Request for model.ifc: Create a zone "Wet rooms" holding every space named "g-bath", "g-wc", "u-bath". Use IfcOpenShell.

First a look at what the model holds.

```python
import ifcopenshell

model = ifcopenshell.open("model.ifc")
print(model.schema)
seen = {}
for space in model.by_type("IfcSpace"):
    seen[space.LongName] = seen.get(space.LongName, 0) + 1
for name, count in sorted(seen.items(), key=str):
    print(count, "x", name)
print("zones:", [z.Name for z in model.by_type("IfcZone")][:20])
```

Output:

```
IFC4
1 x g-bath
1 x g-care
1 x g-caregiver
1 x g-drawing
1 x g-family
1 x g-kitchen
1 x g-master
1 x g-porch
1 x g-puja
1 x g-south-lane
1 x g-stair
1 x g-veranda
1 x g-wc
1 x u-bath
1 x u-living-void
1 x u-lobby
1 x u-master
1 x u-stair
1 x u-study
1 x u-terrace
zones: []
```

```python
import ifcopenshell
import ifcopenshell.api.group
import ifcopenshell.api.root

model = ifcopenshell.open("model.ifc")

names = {"g-bath", "g-wc", "u-bath"}
spaces = [s for s in model.by_type("IfcSpace") if s.LongName in names]

zone = ifcopenshell.api.root.create_entity(model, ifc_class="IfcZone", name="Wet rooms")
ifcopenshell.api.group.assign_group(model, products=spaces, group=zone)
print(len(spaces), "spaces in", zone.Name)

model.write("model_edited.ifc")
```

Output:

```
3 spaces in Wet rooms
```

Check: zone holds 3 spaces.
